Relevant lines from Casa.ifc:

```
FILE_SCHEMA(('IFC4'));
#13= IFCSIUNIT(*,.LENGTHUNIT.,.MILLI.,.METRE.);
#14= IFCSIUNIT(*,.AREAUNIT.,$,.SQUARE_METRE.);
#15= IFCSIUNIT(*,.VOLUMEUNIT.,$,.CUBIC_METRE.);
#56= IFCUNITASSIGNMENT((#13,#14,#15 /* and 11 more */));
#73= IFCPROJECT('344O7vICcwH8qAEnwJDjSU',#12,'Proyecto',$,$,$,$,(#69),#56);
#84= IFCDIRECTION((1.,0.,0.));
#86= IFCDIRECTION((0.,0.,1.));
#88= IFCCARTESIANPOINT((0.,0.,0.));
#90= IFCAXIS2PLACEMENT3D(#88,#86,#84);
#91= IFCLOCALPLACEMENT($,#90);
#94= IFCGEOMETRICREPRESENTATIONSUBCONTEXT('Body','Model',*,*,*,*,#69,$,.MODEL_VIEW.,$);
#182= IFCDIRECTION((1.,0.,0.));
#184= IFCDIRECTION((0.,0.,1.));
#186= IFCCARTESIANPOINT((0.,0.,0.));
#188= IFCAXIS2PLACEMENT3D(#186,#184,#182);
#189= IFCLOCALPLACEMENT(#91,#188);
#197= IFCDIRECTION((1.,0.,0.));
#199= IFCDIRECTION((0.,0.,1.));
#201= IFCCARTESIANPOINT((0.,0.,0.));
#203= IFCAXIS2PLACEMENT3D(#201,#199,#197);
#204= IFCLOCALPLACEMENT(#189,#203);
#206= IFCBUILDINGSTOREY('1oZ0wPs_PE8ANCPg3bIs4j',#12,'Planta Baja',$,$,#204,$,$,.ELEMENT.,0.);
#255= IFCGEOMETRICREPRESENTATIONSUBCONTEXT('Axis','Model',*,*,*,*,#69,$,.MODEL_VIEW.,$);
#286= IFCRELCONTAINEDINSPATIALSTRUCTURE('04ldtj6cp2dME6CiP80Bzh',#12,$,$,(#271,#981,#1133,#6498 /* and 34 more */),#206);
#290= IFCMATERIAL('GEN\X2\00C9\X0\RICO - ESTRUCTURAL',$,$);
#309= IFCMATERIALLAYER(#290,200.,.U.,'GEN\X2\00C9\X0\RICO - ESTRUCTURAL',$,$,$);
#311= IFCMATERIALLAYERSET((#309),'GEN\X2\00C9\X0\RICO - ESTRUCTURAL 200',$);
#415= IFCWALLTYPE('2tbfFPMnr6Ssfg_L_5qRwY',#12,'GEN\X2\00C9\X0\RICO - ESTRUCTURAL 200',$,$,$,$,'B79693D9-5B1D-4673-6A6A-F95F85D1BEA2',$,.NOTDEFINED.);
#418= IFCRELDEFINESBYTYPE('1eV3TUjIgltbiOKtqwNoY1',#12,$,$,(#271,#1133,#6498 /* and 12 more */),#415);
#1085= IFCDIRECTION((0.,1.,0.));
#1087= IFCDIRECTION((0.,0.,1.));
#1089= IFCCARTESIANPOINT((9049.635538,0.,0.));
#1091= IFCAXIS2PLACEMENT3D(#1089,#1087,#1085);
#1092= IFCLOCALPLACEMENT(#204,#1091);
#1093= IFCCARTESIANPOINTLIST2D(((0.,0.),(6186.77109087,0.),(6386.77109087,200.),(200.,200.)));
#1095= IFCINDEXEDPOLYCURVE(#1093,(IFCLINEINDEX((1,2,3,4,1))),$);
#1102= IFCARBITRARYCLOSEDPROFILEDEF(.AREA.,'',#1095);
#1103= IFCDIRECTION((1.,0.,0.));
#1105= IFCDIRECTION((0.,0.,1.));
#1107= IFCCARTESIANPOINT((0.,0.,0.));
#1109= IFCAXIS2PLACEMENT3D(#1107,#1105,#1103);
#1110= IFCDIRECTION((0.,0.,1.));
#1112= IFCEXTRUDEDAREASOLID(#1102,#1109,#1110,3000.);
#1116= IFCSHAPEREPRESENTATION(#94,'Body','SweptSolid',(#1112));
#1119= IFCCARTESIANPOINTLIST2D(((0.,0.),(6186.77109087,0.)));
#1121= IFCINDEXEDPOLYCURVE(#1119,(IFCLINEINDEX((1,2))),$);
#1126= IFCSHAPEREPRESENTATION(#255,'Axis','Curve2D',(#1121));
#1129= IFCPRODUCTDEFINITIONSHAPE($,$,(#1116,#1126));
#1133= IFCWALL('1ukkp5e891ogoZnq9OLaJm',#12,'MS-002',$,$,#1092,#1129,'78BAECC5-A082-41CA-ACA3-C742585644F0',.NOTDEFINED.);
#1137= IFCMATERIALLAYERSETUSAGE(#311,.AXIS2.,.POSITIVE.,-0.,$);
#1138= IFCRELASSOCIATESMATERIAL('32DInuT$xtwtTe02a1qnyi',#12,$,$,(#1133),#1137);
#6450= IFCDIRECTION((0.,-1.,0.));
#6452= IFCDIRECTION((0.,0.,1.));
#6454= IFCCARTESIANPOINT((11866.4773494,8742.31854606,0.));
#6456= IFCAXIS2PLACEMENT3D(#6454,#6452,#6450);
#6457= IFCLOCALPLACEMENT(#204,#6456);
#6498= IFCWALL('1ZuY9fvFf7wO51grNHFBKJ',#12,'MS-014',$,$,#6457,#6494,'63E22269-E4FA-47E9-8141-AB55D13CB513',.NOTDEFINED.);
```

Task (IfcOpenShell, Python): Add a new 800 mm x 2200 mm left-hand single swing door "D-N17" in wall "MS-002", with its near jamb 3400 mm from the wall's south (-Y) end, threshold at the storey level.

```python
import numpy as np
import ifcopenshell
import ifcopenshell.api.feature
import ifcopenshell.api.geometry
import ifcopenshell.api.root
import ifcopenshell.api.spatial
import ifcopenshell.geom
import ifcopenshell.util.element
import ifcopenshell.util.placement
import ifcopenshell.util.representation
import ifcopenshell.util.shape
import ifcopenshell.util.unit

model = ifcopenshell.open("Casa.ifc")
unit_scale = ifcopenshell.util.unit.calculate_unit_scale(model)
settings = ifcopenshell.geom.settings()


def volume(element):
    """Net volume in cubic metres, openings subtracted."""
    shape = ifcopenshell.geom.create_shape(settings, element)
    return ifcopenshell.util.shape.get_volume(shape.geometry)


wall = model.by_guid("1ukkp5e891ogoZnq9OLaJm")
storey = ifcopenshell.util.element.get_container(wall, ifc_class="IfcBuildingStorey")
context = ifcopenshell.util.representation.get_context(model, "Model", "Body", "MODEL_VIEW")
before = volume(wall)

width, height, from_end, sill = 0.8, 2.2, 3.4, 0.0  # metres

# The wall runs along its own X axis, and the end named is its -X end.
wall_shape = ifcopenshell.geom.create_shape(settings, wall)
x, y, z = ifcopenshell.util.shape.get_vertices(wall_shape.geometry).T
start = x.min() + from_end
face, thickness = float(y.min()), float(y.max() - y.min())
wall_matrix = ifcopenshell.util.placement.get_local_placement(wall.ObjectPlacement)
level = ifcopenshell.util.placement.get_local_placement(storey.ObjectPlacement)[2, 3]


def in_wall(x, y):
    """Placement at x, y metres in the wall's axes, at sill height."""
    matrix = wall_matrix.copy()
    matrix[:, 3] = wall_matrix @ np.array([x / unit_scale, y / unit_scale, 0.0, 1.0])
    matrix[2, 3] = level + sill / unit_scale
    return matrix


# Opening: a box that overshoots both wall faces by 50 mm.
opening = ifcopenshell.api.root.create_entity(model, ifc_class="IfcOpeningElement", predefined_type="OPENING")
box = ifcopenshell.api.geometry.add_wall_representation(
    model, context=context, length=width, height=height, thickness=thickness + 0.1
)
ifcopenshell.api.geometry.assign_representation(model, product=opening, representation=box)
ifcopenshell.api.geometry.edit_object_placement(model, product=opening, matrix=in_wall(start, face - 0.05), is_si=False)
ifcopenshell.api.feature.add_feature(model, feature=opening, element=wall)

door = ifcopenshell.api.root.create_entity(model, ifc_class="IfcDoor", name="D-N17", predefined_type="DOOR")
door.OverallWidth, door.OverallHeight = width / unit_scale, height / unit_scale
door.OperationType = "SINGLE_SWING_LEFT"
body = ifcopenshell.api.geometry.add_door_representation(
    model,
    context=context,
    overall_width=door.OverallWidth,
    overall_height=door.OverallHeight,
    operation_type="SINGLE_SWING_LEFT",
    lining_properties={"LiningDepth": thickness / unit_scale, "ThresholdDepth": thickness / unit_scale},
)
ifcopenshell.api.geometry.assign_representation(model, product=door, representation=body)
ifcopenshell.api.spatial.assign_container(model, products=[door], relating_structure=storey)
ifcopenshell.api.feature.add_filling(model, opening=opening, element=door)

# The lining spans the wall, so the door starts at the wall face.
ifcopenshell.api.geometry.edit_object_placement(model, product=door, matrix=in_wall(start, face), is_si=False)

after = volume(wall)

print(f"wall volume {before:.3f} -> {after:.3f} m3")

model.write("Casa_rev.ifc")
```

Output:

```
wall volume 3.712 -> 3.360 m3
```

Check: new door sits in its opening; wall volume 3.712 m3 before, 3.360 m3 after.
